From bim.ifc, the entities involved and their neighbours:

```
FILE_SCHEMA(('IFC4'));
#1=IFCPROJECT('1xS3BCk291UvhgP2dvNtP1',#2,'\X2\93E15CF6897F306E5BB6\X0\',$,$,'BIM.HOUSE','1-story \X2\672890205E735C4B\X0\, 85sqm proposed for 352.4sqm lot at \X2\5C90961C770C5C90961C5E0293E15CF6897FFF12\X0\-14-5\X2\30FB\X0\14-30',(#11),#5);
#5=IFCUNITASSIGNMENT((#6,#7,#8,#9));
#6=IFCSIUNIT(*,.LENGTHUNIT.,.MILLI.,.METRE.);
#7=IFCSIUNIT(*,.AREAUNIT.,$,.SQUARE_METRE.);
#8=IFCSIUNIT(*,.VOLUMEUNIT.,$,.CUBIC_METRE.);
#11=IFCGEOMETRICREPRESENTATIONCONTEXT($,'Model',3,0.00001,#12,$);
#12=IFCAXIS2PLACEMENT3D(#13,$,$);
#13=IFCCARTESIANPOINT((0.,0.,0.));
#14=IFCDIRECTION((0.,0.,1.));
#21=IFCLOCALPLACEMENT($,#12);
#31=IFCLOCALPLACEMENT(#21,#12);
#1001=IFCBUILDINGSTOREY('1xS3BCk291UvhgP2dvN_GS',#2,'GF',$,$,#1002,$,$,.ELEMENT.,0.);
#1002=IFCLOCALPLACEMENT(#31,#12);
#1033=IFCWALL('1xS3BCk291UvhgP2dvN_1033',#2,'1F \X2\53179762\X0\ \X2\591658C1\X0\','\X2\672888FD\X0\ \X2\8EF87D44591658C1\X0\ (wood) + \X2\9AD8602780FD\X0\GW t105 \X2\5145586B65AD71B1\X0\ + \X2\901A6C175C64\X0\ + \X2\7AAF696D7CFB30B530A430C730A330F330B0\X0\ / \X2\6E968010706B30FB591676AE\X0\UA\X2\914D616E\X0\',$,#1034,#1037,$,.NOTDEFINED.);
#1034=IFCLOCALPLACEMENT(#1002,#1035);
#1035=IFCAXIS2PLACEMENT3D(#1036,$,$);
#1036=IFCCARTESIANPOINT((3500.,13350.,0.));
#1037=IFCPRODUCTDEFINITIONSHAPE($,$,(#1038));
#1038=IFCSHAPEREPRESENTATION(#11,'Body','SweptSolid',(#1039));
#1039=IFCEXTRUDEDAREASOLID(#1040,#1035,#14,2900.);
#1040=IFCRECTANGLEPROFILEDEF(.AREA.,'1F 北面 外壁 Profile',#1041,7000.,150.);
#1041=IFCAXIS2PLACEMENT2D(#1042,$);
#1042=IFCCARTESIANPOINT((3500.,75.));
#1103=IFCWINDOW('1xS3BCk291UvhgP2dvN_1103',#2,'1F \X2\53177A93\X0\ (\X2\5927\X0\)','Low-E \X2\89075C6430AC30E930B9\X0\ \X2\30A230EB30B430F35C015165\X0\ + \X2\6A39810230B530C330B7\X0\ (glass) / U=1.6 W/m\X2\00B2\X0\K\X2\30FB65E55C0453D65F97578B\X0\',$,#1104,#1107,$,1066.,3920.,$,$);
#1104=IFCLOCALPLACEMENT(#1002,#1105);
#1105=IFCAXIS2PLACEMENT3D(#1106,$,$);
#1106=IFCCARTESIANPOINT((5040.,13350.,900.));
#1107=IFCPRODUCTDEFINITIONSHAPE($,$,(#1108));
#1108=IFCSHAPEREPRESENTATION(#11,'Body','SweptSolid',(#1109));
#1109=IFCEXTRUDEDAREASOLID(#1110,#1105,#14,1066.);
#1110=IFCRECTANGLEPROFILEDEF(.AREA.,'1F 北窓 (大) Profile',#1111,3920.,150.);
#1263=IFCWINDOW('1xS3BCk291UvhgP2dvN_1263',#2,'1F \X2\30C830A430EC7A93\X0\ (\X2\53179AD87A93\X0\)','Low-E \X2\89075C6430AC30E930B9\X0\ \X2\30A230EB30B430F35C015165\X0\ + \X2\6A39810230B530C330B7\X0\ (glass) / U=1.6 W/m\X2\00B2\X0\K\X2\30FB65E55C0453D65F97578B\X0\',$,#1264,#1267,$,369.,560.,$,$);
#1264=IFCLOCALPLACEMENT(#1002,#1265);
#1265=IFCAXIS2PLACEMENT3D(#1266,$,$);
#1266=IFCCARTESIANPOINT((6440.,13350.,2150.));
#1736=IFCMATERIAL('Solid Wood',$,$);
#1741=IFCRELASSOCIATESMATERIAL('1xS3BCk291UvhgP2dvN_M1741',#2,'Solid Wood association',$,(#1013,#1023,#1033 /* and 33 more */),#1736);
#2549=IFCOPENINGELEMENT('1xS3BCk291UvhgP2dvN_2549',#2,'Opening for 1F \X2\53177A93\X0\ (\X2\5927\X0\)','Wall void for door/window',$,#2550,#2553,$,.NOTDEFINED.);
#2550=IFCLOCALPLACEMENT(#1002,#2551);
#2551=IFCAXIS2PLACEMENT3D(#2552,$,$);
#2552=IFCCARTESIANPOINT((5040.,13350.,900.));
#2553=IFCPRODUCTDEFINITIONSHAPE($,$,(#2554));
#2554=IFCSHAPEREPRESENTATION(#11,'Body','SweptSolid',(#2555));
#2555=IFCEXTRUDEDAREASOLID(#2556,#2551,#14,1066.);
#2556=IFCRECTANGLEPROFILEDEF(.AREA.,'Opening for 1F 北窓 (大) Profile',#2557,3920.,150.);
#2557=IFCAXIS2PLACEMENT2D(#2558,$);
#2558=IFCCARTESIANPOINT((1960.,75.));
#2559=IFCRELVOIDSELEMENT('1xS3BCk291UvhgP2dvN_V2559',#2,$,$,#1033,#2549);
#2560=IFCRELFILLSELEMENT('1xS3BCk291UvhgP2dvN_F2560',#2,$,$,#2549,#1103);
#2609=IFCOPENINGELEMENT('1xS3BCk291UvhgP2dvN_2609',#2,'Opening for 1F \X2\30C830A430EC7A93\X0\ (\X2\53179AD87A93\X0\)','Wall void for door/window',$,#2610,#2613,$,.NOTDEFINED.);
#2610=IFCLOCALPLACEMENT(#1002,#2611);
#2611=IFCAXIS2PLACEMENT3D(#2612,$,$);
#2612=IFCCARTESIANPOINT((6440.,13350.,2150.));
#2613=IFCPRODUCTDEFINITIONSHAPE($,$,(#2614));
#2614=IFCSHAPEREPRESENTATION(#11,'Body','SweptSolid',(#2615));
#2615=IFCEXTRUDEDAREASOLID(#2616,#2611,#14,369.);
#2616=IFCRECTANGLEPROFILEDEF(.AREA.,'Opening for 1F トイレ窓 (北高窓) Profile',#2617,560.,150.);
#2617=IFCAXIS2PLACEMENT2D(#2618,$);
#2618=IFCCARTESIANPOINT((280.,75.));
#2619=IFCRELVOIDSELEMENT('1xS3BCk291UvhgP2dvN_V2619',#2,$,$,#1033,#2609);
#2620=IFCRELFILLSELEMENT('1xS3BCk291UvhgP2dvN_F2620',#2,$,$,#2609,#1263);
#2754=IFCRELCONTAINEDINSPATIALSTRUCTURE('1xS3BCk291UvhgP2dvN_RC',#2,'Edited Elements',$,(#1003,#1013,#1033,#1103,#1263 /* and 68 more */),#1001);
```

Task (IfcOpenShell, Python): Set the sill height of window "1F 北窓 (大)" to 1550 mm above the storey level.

```python
import numpy as np
import ifcopenshell
import ifcopenshell.api.geometry
import ifcopenshell.geom
import ifcopenshell.util.element
import ifcopenshell.util.placement
import ifcopenshell.util.shape
import ifcopenshell.util.unit

model = ifcopenshell.open("bim.ifc")
unit_scale = ifcopenshell.util.unit.calculate_unit_scale(model)

window = model.by_id(1103)
opening = window.FillsVoids[0].RelatingOpeningElement
storey = ifcopenshell.util.element.get_container(window, ifc_class="IfcBuildingStorey")
level = ifcopenshell.util.placement.get_local_placement(storey.ObjectPlacement)[2, 3]

# The opening's origin need not be at the sill, so measure its lowest point.
shape = ifcopenshell.geom.create_shape(ifcopenshell.geom.settings(), opening)
bottom = ifcopenshell.util.shape.get_shape_bottom_elevation(shape, shape.geometry) / unit_scale
dz = level + 1.55 / unit_scale - bottom

shift = np.array([0.0, 0.0, dz])
# The window is not placed relative to its opening, so move both.
for product in (opening, window):
    matrix = ifcopenshell.util.placement.get_local_placement(product.ObjectPlacement)
    matrix[:3, 3] += shift
    ifcopenshell.api.geometry.edit_object_placement(model, product=product, matrix=matrix, is_si=False)

print(f"moved by {dz * unit_scale:+.3f} m")

model.write("bim-out.ifc")
```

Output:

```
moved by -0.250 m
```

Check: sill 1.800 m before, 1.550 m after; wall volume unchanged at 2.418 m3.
